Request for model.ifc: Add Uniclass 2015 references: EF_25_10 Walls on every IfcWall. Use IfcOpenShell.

First a look at what the model holds.

```python
import ifcopenshell

model = ifcopenshell.open("model.ifc")
print(model.schema)
print("classifications:", [c.Name for c in model.by_type("IfcClassification")])
for ifc_class in ("IfcDoor", "IfcRoof", "IfcStair", "IfcWall", "IfcWindow"):
    print(ifc_class, len(model.by_type(ifc_class)))
```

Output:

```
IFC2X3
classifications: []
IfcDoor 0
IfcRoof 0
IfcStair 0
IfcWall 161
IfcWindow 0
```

```python
import ifcopenshell
import ifcopenshell.api.classification

model = ifcopenshell.open("model.ifc")

# IFC2X3 requires Source and Edition and has no link from the project to the system.
system = model.create_entity("IfcClassification", Source="NBS", Edition="2015", Name="Uniclass 2015")

codes = {
    "IfcWall": ("EF_25_10", "Walls"),
}
for ifc_class, (code, name) in codes.items():
    products = model.by_type(ifc_class)
    ifcopenshell.api.classification.add_reference(
        model, products=products, classification=system, identification=code, name=name
    )
    print(code, len(products))

model.write("model_rev.ifc")
```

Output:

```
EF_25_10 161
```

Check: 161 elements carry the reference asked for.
